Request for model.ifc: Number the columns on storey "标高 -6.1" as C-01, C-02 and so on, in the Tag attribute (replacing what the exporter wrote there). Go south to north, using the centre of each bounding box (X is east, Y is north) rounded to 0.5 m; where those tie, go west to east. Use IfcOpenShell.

First a look at what the model holds.

```python
import ifcopenshell
import ifcopenshell.util.element
import ifcopenshell.util.placement

model = ifcopenshell.open("model.ifc")
print(model.schema)
storey = next(s for s in model.by_type("IfcBuildingStorey") if s.Name == "标高 -6.1")
columns = [e for e in ifcopenshell.util.element.get_decomposition(storey) if e.is_a("IfcColumn")]
for e in sorted(columns, key=lambda e: e.id()):
    origin = ifcopenshell.util.placement.get_local_placement(e.ObjectPlacement)[:3, 3]
    print(e.id(), e.Tag, e.Name, origin.round(2) + 0.0, sep=" | ")
```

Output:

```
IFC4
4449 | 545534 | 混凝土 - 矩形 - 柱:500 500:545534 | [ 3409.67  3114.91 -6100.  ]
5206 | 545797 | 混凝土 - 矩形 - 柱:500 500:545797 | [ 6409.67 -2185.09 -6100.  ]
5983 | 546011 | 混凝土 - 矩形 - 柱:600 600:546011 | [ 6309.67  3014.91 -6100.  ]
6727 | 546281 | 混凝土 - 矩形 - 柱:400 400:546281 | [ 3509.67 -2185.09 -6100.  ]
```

```python
import ifcopenshell
import ifcopenshell.geom
import ifcopenshell.util.element
import ifcopenshell.util.shape

model = ifcopenshell.open("model.ifc")
settings = ifcopenshell.geom.settings()
settings.set("use-world-coords", True)


def centre(element):
    shape = ifcopenshell.geom.create_shape(settings, element)
    return ifcopenshell.util.shape.get_bbox_centroid(shape.geometry)


storey = next(s for s in model.by_type("IfcBuildingStorey") if s.Name == "标高 -6.1")
columns = [e for e in ifcopenshell.util.element.get_decomposition(storey) if e.is_a("IfcColumn")]

# Insertion points can sit at a corner or the storey origin, so sort by the geometry (in metres).
centres = {e: centre(e) for e in columns}
columns.sort(key=lambda e: (round(centres[e][1] / 0.5), centres[e][0]))

for i, e in enumerate(columns, start=1):
    number = f"C-{i:02d}"
    e.Tag = number
    print(e.id(), number)

model.write("model_v2.ifc")
```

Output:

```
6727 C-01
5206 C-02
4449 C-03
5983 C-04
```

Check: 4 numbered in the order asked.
